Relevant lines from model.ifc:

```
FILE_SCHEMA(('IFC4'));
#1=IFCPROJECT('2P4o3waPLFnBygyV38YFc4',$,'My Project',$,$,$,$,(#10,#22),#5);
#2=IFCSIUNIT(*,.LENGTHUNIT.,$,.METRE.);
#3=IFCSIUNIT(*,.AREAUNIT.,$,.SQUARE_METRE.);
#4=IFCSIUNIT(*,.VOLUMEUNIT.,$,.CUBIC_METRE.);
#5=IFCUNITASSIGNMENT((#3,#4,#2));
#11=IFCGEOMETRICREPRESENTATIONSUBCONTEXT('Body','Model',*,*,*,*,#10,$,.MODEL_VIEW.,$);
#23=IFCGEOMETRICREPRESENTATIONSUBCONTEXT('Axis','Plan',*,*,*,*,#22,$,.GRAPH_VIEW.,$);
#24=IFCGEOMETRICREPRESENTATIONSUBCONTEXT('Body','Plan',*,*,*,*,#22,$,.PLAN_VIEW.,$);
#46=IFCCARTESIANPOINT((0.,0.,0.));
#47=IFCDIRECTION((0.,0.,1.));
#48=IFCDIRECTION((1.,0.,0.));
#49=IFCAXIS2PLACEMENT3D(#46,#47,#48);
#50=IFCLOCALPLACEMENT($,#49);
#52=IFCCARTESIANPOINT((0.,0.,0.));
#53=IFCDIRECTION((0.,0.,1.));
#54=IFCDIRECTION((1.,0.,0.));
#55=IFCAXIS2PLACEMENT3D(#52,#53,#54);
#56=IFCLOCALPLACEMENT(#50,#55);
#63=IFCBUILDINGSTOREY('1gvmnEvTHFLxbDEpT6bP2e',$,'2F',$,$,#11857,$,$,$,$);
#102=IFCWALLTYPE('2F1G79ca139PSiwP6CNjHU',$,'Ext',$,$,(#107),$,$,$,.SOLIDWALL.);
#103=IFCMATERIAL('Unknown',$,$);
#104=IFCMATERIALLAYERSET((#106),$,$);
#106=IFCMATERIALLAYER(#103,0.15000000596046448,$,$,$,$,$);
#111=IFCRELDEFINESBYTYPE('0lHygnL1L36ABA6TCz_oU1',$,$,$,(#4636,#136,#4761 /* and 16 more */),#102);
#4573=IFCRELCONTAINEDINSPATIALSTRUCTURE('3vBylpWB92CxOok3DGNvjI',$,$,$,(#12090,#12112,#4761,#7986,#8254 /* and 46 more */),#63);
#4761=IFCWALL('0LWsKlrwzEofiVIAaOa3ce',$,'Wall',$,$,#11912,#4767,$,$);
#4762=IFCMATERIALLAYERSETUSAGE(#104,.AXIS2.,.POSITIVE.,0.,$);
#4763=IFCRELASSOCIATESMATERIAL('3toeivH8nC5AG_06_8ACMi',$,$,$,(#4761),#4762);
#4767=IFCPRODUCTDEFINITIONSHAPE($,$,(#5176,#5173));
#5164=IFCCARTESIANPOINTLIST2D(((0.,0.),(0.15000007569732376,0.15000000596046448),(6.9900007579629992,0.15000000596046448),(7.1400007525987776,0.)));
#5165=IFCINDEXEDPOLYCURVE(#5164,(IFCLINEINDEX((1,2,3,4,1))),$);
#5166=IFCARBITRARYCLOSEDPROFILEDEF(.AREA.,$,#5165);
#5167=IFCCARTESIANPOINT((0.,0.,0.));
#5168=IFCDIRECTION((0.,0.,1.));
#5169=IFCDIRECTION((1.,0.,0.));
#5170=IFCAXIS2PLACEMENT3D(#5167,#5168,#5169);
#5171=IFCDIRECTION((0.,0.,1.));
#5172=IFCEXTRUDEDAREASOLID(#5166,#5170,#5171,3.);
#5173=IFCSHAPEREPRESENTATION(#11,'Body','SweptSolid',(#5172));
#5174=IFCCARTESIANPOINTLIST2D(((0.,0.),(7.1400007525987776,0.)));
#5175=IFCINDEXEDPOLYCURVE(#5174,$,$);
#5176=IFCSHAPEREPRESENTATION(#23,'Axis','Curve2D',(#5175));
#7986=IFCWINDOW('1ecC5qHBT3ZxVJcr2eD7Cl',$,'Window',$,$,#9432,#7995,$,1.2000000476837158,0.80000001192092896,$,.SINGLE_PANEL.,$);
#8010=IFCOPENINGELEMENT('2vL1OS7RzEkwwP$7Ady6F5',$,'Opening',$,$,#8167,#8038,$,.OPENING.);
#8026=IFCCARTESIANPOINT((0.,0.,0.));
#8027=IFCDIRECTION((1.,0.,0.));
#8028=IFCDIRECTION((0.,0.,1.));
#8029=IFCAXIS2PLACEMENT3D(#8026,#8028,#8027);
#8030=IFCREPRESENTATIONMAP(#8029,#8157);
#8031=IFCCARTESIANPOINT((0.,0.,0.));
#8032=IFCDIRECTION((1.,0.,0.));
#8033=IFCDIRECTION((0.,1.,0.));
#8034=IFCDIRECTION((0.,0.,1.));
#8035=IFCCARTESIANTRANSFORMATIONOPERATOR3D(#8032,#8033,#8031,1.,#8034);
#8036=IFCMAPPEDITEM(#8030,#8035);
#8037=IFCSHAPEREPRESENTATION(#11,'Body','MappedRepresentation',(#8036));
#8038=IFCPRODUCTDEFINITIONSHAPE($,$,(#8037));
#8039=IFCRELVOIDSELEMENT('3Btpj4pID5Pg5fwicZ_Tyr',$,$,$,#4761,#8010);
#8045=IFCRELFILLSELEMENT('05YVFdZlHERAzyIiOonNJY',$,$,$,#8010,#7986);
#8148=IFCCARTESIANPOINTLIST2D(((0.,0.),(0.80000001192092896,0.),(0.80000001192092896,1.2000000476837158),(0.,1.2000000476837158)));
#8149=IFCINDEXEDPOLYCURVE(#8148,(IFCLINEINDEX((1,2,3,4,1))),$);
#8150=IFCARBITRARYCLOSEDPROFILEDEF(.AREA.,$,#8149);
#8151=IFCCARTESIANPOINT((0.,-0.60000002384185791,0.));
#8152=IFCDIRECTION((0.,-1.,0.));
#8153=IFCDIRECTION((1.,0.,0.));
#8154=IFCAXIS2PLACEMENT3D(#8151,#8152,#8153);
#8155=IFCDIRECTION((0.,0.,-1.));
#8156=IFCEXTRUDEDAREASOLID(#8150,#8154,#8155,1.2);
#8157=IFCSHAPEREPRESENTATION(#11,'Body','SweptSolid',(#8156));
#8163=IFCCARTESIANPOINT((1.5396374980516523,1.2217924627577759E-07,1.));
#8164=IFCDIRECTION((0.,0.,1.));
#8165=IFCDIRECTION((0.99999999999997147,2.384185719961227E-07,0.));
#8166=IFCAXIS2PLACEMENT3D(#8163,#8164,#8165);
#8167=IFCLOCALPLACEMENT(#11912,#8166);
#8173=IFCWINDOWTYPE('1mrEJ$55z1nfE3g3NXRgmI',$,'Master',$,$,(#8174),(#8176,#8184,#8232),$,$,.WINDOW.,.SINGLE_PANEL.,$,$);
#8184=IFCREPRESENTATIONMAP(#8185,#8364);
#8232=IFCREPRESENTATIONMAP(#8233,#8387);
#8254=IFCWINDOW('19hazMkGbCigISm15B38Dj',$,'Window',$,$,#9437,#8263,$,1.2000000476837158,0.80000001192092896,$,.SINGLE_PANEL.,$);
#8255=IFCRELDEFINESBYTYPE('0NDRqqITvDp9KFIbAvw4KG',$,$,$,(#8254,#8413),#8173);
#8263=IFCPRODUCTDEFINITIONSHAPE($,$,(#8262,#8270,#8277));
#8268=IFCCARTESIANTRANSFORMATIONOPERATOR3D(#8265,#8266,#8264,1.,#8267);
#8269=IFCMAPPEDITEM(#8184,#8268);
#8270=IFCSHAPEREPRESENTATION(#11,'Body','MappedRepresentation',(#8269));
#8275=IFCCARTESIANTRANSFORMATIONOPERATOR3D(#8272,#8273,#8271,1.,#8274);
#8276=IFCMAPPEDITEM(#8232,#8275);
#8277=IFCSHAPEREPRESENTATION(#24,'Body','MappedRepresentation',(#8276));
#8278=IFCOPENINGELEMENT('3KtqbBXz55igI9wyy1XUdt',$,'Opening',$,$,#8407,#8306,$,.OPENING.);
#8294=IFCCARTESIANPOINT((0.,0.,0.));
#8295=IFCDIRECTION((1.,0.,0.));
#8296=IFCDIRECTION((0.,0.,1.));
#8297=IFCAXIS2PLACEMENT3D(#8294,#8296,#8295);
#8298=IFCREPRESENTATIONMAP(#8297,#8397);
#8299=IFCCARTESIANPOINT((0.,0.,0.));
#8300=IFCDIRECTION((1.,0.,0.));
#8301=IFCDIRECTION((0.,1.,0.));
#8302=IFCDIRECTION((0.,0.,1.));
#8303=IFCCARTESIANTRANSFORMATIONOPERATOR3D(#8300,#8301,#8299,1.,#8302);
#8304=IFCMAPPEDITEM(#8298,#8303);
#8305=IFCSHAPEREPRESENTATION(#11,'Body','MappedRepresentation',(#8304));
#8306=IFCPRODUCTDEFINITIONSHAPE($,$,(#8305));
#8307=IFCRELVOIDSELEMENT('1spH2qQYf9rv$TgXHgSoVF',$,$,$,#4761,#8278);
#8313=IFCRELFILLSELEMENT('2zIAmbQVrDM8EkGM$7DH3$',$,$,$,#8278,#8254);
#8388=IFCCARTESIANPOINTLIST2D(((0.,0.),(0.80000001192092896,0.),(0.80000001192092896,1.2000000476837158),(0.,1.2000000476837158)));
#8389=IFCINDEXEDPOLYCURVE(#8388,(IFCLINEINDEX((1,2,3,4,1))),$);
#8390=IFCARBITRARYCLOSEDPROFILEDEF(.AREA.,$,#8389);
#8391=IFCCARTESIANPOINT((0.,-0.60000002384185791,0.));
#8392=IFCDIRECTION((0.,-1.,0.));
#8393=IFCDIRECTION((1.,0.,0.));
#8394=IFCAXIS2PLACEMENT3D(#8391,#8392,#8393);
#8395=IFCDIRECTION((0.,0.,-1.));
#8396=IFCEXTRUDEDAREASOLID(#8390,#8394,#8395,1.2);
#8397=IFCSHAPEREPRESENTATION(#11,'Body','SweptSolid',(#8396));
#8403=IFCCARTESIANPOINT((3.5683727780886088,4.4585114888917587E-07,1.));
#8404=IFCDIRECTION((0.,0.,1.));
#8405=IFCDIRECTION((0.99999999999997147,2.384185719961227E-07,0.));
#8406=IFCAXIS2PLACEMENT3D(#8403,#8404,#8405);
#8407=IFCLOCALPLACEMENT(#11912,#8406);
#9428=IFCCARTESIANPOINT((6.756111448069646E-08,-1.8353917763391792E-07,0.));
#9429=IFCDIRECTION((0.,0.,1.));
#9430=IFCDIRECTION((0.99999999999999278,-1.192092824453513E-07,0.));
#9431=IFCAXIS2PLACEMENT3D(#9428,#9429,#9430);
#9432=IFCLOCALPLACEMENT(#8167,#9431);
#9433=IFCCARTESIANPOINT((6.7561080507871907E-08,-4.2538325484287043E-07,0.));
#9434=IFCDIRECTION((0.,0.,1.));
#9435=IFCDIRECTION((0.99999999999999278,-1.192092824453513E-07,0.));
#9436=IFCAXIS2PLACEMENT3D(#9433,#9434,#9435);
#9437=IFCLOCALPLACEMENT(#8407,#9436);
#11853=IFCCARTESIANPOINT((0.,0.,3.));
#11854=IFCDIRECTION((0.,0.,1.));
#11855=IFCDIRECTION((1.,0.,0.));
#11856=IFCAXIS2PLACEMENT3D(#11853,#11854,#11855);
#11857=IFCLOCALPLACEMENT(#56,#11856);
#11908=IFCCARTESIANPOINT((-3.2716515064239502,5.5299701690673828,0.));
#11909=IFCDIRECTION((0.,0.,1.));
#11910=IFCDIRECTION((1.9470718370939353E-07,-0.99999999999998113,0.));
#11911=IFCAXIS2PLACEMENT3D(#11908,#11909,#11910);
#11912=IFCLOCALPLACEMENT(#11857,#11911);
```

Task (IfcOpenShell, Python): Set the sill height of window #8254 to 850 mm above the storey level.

```python
import numpy as np
import ifcopenshell
import ifcopenshell.api.geometry
import ifcopenshell.geom
import ifcopenshell.util.element
import ifcopenshell.util.placement
import ifcopenshell.util.shape
import ifcopenshell.util.unit

model = ifcopenshell.open("model.ifc")
unit_scale = ifcopenshell.util.unit.calculate_unit_scale(model)

window = model.by_guid("19hazMkGbCigISm15B38Dj")
opening = window.FillsVoids[0].RelatingOpeningElement
storey = ifcopenshell.util.element.get_container(window, ifc_class="IfcBuildingStorey")
level = ifcopenshell.util.placement.get_local_placement(storey.ObjectPlacement)[2, 3]

# The opening's origin need not be at the sill, so measure its lowest point.
shape = ifcopenshell.geom.create_shape(ifcopenshell.geom.settings(), opening)
bottom = ifcopenshell.util.shape.get_shape_bottom_elevation(shape, shape.geometry) / unit_scale
dz = level + 0.85 / unit_scale - bottom

shift = np.array([0.0, 0.0, dz])
# The window is placed relative to its opening, so it follows when the opening moves.
matrix = ifcopenshell.util.placement.get_local_placement(opening.ObjectPlacement)
matrix[:3, 3] += shift
ifcopenshell.api.geometry.edit_object_placement(
    model, product=opening, matrix=matrix, is_si=False, should_transform_children=True
)

print(f"moved by {dz * unit_scale:+.3f} m")

model.write("model-out.ifc")
```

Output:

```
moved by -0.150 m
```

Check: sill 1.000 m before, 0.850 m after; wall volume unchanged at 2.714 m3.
